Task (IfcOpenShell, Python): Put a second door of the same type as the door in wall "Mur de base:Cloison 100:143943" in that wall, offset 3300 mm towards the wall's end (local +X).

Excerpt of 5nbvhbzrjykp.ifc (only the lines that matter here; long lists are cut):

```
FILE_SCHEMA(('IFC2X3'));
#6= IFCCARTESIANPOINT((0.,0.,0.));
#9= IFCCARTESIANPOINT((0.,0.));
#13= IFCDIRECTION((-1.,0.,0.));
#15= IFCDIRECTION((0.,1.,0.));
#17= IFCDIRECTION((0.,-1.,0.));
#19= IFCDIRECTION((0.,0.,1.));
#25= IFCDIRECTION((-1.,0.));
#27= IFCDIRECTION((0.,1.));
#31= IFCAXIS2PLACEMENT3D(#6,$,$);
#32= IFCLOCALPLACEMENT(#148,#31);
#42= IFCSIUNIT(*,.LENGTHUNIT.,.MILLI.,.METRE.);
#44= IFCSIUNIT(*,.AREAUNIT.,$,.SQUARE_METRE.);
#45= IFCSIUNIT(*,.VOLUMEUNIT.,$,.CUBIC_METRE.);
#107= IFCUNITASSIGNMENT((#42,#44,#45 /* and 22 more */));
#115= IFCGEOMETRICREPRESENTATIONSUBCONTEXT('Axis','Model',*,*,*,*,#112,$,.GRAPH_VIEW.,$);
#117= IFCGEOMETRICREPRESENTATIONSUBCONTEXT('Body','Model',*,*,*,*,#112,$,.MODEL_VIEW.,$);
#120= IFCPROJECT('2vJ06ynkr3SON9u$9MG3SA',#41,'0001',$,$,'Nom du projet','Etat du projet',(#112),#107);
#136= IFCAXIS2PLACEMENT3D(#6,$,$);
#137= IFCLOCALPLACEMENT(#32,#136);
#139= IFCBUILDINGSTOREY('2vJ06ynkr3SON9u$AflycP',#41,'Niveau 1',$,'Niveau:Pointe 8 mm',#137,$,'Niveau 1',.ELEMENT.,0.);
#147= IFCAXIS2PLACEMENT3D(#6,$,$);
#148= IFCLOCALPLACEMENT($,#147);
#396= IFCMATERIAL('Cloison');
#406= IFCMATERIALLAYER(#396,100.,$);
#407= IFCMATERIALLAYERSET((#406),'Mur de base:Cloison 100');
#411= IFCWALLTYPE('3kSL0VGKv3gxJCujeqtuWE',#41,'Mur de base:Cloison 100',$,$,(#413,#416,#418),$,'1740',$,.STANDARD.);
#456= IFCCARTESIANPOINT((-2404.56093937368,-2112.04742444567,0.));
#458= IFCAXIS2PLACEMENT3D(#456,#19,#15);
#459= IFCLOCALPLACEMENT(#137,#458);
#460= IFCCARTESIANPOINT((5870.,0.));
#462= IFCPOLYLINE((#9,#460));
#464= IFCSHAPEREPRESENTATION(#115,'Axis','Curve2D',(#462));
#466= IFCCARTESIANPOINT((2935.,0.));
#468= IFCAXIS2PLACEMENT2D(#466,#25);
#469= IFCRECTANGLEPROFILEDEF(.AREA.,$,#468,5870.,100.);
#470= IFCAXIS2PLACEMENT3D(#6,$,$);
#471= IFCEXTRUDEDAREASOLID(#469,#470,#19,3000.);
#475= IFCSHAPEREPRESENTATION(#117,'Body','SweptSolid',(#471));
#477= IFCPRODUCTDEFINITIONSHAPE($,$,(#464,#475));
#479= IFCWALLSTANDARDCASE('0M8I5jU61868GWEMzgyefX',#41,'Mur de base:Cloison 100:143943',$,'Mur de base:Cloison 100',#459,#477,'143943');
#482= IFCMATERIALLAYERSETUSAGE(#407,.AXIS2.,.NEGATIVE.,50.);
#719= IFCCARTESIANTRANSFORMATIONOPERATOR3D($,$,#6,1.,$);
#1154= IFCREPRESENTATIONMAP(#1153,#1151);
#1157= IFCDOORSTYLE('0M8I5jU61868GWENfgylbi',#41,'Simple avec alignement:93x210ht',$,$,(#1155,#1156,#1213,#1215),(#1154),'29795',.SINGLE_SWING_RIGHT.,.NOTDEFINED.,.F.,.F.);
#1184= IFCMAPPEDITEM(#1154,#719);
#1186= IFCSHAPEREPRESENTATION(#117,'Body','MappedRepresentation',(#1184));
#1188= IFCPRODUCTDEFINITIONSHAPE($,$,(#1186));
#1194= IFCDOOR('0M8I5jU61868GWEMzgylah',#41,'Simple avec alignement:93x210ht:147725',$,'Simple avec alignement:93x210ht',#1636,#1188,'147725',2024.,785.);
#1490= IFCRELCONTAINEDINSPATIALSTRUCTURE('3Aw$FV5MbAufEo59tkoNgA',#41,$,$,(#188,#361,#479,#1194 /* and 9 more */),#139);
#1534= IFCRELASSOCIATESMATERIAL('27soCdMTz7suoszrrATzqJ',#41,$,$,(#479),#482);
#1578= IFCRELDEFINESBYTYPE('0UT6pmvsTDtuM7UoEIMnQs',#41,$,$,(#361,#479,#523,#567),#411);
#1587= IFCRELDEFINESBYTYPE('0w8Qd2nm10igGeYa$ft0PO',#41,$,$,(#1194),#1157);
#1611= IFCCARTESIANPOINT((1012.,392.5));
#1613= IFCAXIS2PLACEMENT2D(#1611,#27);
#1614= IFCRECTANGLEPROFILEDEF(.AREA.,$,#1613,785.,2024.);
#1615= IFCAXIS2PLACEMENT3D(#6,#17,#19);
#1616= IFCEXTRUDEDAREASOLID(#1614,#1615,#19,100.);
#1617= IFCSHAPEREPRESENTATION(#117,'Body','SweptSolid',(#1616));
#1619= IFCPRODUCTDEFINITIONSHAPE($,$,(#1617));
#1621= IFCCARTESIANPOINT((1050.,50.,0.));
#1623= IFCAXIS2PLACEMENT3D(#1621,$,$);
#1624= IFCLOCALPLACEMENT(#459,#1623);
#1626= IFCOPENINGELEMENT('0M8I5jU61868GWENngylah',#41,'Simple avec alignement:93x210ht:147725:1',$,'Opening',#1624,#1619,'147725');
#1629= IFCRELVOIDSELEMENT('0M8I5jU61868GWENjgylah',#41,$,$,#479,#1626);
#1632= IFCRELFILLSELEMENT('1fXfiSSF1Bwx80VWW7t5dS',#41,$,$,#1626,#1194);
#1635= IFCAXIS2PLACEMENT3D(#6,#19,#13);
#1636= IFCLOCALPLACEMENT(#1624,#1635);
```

```python
import ifcopenshell
import ifcopenshell.api.feature
import ifcopenshell.api.geometry
import ifcopenshell.api.root
import ifcopenshell.geom
import ifcopenshell.util.element
import ifcopenshell.util.placement
import ifcopenshell.util.shape

model = ifcopenshell.open("5nbvhbzrjykp.ifc")
settings = ifcopenshell.geom.settings()


def volume(element):
    """Net volume in cubic metres, openings subtracted."""
    shape = ifcopenshell.geom.create_shape(settings, element)
    return ifcopenshell.util.shape.get_volume(shape.geometry)


def reuse_history(source, copy):
    """copy_class also copies each property set's owner history, people and application; keep the originals."""
    for rel in copy.IsDefinedBy:
        if rel.is_a("IfcRelDefinesByProperties") and (history := rel.RelatingPropertyDefinition.OwnerHistory):
            rel.RelatingPropertyDefinition.OwnerHistory = source.OwnerHistory
            ifcopenshell.util.element.remove_deep2(model, history)


door = model.by_id(1194)
opening = door.FillsVoids[0].RelatingOpeningElement
wall = opening.VoidsElements[0].RelatingBuildingElement
before = volume(wall)
shift = ifcopenshell.util.placement.get_local_placement(wall.ObjectPlacement)[:3, 0] * 3300.0

# copy_class copies the void relationship, type, container and properties, but no geometry.
new_opening = ifcopenshell.api.root.copy_class(model, product=opening)
new_opening.Representation = ifcopenshell.util.element.copy_deep(
    model, opening.Representation, exclude=["IfcGeometricRepresentationContext", "IfcRepresentationMap"]
)
new_opening.Name = "Simple avec alignement:93x210ht"
new_opening.Tag = None
new_door = ifcopenshell.api.root.copy_class(model, product=door)
new_door.Representation = ifcopenshell.util.element.copy_deep(
    model, door.Representation, exclude=["IfcGeometricRepresentationContext", "IfcRepresentationMap"]
)
new_door.Name = "Simple avec alignement:93x210ht"
new_door.Tag = None
reuse_history(door, new_door)
fills = ifcopenshell.api.feature.add_filling(model, opening=new_opening, element=new_door)
fills.OwnerHistory = new_door.OwnerHistory  # required in IFC2X3

for old, new in ((opening, new_opening), (door, new_door)):
    matrix = ifcopenshell.util.placement.get_local_placement(old.ObjectPlacement)
    matrix[:3, 3] += shift
    ifcopenshell.api.geometry.edit_object_placement(model, product=new, matrix=matrix, is_si=False)

after = volume(wall)

print(f"wall volume {before:.3f} -> {after:.3f} m3")

model.write("5nbvhbzrjykp_updated.ifc")
```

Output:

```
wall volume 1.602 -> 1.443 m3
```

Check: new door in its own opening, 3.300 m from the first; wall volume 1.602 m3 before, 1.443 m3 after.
